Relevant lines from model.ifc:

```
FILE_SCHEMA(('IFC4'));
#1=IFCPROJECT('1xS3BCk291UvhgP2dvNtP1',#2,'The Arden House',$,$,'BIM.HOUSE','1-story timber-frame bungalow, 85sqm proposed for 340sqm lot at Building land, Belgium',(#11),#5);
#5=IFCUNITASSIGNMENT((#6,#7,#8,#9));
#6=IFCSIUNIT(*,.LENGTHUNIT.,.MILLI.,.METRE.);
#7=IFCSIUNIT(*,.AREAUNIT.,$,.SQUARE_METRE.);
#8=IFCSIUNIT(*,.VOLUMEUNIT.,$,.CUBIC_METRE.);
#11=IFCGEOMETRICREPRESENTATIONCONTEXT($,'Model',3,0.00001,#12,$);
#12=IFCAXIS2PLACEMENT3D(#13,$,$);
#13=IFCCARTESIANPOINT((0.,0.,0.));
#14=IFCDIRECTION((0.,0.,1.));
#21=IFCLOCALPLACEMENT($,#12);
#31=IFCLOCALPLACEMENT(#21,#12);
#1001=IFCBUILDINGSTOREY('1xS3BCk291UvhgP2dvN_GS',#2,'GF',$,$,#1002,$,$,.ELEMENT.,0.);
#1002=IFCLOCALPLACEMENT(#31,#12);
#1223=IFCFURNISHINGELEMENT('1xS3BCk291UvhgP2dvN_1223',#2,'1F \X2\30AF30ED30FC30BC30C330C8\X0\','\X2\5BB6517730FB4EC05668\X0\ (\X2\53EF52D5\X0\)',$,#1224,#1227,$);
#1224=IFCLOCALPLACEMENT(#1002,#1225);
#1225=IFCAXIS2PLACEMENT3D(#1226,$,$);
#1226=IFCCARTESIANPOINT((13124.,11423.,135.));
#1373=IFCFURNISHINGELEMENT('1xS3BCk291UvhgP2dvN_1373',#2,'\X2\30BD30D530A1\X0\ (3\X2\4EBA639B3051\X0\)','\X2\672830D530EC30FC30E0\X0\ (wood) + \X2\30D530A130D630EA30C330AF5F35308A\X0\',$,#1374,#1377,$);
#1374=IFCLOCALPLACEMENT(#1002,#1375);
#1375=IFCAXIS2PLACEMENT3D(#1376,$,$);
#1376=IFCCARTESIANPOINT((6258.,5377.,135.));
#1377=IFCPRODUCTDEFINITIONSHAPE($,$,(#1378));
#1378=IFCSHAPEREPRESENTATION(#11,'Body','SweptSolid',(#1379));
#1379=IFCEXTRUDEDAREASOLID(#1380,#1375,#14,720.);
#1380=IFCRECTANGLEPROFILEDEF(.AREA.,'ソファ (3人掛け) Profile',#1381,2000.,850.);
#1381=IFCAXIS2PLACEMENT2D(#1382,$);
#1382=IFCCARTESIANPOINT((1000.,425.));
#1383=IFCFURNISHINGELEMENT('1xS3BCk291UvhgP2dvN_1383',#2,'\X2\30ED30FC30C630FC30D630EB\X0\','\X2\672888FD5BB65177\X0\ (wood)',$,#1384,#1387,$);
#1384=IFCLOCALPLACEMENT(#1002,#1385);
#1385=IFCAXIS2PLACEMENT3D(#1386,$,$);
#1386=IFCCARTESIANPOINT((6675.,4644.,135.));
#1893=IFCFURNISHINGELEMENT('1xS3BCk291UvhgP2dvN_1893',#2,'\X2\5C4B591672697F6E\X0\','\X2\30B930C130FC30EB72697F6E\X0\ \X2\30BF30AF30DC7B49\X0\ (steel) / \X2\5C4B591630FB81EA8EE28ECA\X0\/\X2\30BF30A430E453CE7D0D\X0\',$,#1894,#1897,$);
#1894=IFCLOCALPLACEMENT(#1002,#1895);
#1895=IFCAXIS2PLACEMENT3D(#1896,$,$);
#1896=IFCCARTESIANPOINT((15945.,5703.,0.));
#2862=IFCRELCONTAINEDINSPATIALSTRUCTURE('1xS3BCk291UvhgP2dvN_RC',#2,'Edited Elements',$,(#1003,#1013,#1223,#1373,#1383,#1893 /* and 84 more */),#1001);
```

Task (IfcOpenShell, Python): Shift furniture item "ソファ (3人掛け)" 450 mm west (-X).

```python
import ifcopenshell
import ifcopenshell.api.geometry
import ifcopenshell.util.placement
import ifcopenshell.util.unit

model = ifcopenshell.open("model.ifc")
unit_scale = ifcopenshell.util.unit.calculate_unit_scale(model)

item = model.by_id(1373)
matrix = ifcopenshell.util.placement.get_local_placement(item.ObjectPlacement)
matrix[0, 3] -= 0.45 / unit_scale
ifcopenshell.api.geometry.edit_object_placement(model, product=item, matrix=matrix, is_si=False)

print(ifcopenshell.util.placement.get_local_placement(item.ObjectPlacement).round(3) + 0.0)

model.write("model_updated.ifc")
```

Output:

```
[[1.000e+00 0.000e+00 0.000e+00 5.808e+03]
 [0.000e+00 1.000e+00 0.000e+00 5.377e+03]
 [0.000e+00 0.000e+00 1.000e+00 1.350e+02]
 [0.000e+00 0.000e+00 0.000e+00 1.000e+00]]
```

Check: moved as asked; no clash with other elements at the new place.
